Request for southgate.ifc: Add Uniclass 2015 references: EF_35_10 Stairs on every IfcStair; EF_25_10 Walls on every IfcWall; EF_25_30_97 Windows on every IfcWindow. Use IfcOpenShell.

First a look at what the model holds.

```python
import ifcopenshell

model = ifcopenshell.open("southgate.ifc")
print(model.schema)
print("classifications:", [c.Name for c in model.by_type("IfcClassification")])
for ifc_class in ("IfcDoor", "IfcRoof", "IfcStair", "IfcWall", "IfcWindow"):
    print(ifc_class, len(model.by_type(ifc_class)))
```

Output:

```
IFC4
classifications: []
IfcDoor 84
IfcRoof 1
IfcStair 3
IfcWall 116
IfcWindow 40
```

```python
import ifcopenshell
import ifcopenshell.api.classification

model = ifcopenshell.open("southgate.ifc")

system = ifcopenshell.api.classification.add_classification(model, classification="Uniclass 2015")

codes = {
    "IfcStair": ("EF_35_10", "Stairs"),
    "IfcWall": ("EF_25_10", "Walls"),
    "IfcWindow": ("EF_25_30_97", "Windows"),
}
for ifc_class, (code, name) in codes.items():
    products = model.by_type(ifc_class)
    ifcopenshell.api.classification.add_reference(
        model, products=products, classification=system, identification=code, name=name
    )
    print(code, len(products))

model.write("southgate_edited.ifc")
```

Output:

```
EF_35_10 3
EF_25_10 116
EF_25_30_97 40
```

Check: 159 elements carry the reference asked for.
